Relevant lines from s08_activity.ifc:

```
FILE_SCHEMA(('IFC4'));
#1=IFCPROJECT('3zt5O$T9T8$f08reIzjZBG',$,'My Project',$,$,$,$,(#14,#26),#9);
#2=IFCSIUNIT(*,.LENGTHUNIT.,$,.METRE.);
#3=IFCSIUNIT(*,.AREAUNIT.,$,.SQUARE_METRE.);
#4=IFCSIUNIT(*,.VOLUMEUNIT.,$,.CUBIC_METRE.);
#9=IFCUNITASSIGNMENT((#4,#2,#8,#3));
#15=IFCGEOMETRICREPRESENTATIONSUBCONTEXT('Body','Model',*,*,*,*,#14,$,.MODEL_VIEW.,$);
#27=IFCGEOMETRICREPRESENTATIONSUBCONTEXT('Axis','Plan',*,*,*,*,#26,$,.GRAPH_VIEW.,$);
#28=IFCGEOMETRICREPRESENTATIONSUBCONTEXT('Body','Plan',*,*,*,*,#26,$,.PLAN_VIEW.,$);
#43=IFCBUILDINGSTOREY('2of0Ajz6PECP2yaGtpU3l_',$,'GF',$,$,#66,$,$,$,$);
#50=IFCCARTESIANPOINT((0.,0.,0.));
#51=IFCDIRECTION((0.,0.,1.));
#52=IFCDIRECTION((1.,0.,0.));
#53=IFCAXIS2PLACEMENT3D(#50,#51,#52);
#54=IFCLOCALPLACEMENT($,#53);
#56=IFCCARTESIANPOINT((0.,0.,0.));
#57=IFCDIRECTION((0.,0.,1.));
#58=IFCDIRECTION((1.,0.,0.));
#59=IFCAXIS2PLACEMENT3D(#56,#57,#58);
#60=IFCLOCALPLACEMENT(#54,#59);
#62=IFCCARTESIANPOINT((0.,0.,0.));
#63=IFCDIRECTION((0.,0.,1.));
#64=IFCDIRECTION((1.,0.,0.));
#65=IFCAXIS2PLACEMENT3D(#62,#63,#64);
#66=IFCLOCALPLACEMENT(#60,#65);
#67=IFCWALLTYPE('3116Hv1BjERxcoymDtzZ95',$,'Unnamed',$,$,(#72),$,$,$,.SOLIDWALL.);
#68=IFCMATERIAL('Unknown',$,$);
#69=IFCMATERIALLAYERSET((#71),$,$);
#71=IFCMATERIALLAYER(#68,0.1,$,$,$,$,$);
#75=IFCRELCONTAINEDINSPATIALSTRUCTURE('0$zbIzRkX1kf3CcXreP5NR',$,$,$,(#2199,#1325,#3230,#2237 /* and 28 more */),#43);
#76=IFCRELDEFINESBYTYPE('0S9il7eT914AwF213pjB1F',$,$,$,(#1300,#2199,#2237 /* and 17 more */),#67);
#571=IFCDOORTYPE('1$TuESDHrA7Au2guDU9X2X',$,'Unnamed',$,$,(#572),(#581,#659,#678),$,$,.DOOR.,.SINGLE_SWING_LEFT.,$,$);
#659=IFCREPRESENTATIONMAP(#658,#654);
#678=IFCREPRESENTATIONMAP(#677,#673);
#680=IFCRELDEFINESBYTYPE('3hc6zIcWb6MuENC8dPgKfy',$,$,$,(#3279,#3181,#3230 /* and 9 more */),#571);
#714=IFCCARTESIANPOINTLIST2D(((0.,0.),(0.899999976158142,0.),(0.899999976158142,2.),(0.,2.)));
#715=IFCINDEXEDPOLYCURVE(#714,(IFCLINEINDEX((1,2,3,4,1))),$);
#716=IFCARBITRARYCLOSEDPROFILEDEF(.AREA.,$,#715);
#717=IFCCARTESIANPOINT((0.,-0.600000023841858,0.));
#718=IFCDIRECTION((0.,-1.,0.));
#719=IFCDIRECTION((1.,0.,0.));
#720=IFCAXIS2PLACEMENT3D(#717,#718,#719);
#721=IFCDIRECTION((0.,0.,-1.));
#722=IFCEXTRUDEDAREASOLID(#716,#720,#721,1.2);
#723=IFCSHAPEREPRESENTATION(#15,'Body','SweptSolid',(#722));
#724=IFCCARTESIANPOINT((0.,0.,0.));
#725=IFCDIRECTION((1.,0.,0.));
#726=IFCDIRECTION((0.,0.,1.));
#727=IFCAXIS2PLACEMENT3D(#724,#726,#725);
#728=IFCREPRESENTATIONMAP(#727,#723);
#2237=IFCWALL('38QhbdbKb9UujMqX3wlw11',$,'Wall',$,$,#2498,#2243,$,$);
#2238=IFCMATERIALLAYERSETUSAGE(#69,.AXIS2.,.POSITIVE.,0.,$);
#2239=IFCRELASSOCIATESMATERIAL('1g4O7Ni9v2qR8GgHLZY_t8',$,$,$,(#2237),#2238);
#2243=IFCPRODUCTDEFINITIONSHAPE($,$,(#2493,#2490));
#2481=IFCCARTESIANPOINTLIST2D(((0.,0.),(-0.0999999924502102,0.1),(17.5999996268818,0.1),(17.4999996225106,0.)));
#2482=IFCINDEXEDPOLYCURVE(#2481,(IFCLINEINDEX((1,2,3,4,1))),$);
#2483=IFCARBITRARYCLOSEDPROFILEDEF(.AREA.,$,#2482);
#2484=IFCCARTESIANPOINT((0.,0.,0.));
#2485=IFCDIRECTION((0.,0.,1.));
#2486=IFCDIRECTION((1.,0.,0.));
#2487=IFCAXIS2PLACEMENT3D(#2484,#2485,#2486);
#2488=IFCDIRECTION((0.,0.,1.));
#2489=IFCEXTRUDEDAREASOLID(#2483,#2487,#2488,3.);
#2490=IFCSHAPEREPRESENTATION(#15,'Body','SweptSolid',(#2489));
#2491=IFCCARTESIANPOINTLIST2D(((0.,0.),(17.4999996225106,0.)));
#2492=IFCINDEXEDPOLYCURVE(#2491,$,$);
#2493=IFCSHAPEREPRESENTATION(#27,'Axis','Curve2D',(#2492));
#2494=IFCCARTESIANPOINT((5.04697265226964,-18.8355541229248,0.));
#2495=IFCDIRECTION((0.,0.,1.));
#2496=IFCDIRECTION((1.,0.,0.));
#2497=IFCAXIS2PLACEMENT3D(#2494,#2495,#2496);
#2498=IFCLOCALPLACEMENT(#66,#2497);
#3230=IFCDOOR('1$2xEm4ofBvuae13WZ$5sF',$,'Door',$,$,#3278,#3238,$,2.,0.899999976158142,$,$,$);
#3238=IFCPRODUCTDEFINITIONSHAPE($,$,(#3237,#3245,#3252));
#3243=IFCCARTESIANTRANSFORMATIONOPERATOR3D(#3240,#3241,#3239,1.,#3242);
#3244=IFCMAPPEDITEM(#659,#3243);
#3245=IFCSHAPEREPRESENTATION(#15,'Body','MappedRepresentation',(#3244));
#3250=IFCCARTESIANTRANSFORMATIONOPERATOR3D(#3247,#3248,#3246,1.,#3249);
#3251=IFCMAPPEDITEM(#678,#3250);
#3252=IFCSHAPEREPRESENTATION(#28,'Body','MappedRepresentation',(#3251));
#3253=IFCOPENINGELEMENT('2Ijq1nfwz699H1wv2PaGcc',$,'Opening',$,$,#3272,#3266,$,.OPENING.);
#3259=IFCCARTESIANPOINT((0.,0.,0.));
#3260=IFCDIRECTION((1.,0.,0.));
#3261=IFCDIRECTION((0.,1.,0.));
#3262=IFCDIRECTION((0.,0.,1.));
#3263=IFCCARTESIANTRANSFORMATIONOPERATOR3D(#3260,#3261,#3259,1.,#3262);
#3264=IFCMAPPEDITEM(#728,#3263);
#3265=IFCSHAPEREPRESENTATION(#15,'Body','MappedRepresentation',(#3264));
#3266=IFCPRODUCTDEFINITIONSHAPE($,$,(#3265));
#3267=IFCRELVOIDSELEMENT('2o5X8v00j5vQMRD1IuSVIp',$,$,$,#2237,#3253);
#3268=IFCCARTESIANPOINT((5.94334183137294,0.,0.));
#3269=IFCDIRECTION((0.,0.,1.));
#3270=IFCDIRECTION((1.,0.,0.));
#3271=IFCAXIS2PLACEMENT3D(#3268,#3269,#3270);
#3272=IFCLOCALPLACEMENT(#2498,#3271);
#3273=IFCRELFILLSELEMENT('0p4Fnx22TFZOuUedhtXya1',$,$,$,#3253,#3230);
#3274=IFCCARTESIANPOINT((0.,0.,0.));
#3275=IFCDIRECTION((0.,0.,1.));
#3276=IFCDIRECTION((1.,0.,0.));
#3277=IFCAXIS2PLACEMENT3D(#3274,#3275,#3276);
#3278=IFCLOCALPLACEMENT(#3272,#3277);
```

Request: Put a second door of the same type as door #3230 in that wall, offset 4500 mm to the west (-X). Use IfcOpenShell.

```python
import ifcopenshell
import ifcopenshell.api.feature
import ifcopenshell.api.geometry
import ifcopenshell.api.root
import ifcopenshell.geom
import ifcopenshell.util.element
import ifcopenshell.util.placement
import ifcopenshell.util.shape

model = ifcopenshell.open("s08_activity.ifc")
settings = ifcopenshell.geom.settings()


def volume(element):
    """Net volume in cubic metres, openings subtracted."""
    shape = ifcopenshell.geom.create_shape(settings, element)
    return ifcopenshell.util.shape.get_volume(shape.geometry)


door = model.by_guid("1$2xEm4ofBvuae13WZ$5sF")
opening = door.FillsVoids[0].RelatingOpeningElement
wall = opening.VoidsElements[0].RelatingBuildingElement
before = volume(wall)
shift = ifcopenshell.util.placement.get_local_placement(wall.ObjectPlacement)[:3, 0] * -4.5

# copy_class copies the void relationship, type, container and properties, but no geometry.
new_opening = ifcopenshell.api.root.copy_class(model, product=opening)
new_opening.Representation = ifcopenshell.util.element.copy_deep(
    model, opening.Representation, exclude=["IfcGeometricRepresentationContext", "IfcRepresentationMap"]
)
new_door = ifcopenshell.api.root.copy_class(model, product=door)
new_door.Representation = ifcopenshell.util.element.copy_deep(
    model, door.Representation, exclude=["IfcGeometricRepresentationContext", "IfcRepresentationMap"]
)
ifcopenshell.api.feature.add_filling(model, opening=new_opening, element=new_door)

for old, new in ((opening, new_opening), (door, new_door)):
    matrix = ifcopenshell.util.placement.get_local_placement(old.ObjectPlacement)
    matrix[:3, 3] += shift
    ifcopenshell.api.geometry.edit_object_placement(model, product=new, matrix=matrix, is_si=False)

after = volume(wall)

print(f"wall volume {before:.3f} -> {after:.3f} m3")

model.write("s08_activity_updated.ifc")
```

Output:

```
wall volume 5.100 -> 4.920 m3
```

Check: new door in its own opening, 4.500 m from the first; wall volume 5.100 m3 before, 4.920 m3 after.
